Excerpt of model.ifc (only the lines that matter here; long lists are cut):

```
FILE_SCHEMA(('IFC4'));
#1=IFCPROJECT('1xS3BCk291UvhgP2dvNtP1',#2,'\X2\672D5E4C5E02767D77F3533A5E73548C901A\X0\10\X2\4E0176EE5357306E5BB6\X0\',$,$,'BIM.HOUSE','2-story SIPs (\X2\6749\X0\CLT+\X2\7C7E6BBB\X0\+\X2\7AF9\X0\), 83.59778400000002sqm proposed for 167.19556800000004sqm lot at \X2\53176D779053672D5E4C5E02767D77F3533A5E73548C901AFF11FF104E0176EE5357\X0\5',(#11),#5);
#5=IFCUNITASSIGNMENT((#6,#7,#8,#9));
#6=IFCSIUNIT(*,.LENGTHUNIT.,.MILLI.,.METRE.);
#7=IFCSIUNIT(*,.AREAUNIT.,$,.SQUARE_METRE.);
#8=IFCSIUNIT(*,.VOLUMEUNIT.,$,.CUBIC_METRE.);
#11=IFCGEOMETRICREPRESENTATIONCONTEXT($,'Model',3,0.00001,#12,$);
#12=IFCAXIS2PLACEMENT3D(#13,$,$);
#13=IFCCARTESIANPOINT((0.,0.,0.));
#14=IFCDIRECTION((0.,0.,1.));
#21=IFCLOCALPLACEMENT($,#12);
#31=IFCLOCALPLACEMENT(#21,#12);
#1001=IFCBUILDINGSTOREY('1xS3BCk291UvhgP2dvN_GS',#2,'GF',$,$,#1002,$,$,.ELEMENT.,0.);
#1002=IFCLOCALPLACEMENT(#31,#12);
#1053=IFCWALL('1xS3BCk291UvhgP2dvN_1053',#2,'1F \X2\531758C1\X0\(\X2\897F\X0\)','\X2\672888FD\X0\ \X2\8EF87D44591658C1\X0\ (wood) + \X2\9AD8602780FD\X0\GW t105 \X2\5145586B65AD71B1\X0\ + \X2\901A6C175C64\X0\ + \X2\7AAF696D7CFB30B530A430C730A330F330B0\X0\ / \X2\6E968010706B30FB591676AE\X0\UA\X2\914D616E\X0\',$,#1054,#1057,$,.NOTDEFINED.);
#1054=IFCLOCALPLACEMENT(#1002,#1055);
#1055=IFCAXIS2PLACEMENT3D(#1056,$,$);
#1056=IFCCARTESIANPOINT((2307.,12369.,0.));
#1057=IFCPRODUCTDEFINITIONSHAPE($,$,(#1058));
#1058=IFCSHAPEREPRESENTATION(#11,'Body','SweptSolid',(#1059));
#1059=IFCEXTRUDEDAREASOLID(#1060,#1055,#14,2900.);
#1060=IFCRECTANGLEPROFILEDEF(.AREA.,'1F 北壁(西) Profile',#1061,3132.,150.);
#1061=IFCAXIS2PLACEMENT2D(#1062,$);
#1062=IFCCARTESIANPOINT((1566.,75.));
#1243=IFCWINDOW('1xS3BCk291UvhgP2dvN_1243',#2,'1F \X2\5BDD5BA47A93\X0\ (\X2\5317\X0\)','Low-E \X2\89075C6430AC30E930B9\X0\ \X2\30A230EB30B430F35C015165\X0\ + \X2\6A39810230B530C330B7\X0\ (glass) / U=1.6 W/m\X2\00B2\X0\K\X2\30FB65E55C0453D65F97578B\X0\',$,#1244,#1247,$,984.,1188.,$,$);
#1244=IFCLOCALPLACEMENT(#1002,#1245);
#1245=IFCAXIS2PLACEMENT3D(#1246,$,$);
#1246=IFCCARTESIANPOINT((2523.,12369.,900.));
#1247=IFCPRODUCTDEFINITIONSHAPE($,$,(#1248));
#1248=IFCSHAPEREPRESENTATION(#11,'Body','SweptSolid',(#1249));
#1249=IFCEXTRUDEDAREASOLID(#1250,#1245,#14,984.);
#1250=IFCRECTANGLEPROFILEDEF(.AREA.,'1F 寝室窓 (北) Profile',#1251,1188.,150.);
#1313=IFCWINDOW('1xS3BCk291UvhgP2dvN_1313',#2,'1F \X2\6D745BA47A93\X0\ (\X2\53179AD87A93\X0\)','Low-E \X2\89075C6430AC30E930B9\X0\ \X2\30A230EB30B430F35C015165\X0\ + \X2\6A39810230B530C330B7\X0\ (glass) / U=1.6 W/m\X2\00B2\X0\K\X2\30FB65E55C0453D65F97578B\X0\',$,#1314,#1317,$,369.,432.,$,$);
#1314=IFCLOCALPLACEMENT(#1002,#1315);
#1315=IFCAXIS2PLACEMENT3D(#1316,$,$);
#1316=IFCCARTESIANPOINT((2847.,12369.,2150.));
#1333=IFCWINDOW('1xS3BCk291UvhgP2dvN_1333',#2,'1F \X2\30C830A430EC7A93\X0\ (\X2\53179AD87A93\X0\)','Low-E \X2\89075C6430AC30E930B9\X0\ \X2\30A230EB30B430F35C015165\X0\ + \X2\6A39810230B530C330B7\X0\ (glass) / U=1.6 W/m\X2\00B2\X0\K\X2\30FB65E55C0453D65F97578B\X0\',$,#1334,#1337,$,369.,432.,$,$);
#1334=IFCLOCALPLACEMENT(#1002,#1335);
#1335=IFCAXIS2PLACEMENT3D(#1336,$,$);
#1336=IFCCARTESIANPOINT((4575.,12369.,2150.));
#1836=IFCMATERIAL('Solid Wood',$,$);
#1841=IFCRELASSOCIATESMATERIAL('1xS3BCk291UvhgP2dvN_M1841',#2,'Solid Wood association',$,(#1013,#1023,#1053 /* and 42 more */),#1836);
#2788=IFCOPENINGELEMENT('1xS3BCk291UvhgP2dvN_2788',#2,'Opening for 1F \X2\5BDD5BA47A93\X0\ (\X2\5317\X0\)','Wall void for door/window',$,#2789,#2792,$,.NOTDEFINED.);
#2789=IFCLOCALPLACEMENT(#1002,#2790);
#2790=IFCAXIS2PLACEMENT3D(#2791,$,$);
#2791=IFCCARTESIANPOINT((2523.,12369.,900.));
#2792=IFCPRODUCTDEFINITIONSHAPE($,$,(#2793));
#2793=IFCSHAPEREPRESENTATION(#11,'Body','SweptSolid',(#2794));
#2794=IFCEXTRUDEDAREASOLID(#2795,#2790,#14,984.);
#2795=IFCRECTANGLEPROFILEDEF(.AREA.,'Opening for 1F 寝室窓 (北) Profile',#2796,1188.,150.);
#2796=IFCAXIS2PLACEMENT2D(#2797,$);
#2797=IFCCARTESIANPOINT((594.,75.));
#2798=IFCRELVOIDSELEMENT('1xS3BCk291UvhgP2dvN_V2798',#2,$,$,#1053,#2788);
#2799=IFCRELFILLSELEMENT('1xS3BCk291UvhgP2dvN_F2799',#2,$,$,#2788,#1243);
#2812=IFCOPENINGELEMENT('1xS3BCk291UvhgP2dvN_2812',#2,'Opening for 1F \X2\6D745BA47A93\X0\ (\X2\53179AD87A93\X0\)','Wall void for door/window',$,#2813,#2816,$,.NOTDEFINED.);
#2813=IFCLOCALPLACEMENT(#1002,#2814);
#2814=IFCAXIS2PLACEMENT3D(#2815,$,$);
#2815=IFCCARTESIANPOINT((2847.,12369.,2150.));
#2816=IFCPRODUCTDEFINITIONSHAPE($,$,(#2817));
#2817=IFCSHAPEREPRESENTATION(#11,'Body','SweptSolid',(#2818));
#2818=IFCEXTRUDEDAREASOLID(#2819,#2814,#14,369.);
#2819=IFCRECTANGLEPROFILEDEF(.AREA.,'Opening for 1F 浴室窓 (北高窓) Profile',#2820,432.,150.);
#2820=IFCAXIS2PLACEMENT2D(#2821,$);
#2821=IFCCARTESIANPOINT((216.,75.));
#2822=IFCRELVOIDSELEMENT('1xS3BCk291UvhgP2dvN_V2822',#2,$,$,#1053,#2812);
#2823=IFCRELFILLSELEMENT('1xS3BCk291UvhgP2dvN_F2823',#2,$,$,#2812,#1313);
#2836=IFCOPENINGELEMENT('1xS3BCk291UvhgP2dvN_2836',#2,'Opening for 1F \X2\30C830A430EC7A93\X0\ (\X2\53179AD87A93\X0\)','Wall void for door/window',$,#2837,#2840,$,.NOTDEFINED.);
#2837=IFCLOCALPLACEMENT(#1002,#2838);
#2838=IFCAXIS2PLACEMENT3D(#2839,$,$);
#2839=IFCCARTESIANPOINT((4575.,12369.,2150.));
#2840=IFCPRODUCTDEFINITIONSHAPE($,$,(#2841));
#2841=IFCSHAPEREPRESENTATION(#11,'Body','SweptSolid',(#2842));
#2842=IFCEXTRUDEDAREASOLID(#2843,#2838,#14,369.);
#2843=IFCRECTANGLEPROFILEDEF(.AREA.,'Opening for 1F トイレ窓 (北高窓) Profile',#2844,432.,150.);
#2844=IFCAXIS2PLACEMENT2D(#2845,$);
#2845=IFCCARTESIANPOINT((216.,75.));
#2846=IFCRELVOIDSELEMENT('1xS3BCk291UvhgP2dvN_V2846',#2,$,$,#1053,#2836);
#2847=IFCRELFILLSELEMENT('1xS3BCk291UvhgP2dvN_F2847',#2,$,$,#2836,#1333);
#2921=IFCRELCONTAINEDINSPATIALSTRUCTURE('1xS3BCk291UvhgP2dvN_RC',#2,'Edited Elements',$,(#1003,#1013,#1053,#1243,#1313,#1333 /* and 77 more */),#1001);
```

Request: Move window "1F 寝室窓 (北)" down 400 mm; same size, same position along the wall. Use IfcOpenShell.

```python
import numpy as np
import ifcopenshell
import ifcopenshell.api.geometry
import ifcopenshell.util.placement
import ifcopenshell.util.unit

model = ifcopenshell.open("model.ifc")
unit_scale = ifcopenshell.util.unit.calculate_unit_scale(model)

window = model.by_id(1243)
opening = window.FillsVoids[0].RelatingOpeningElement
dz = -0.4 / unit_scale

shift = np.array([0.0, 0.0, dz])
# The window is not placed relative to its opening, so move both.
for product in (opening, window):
    matrix = ifcopenshell.util.placement.get_local_placement(product.ObjectPlacement)
    matrix[:3, 3] += shift
    ifcopenshell.api.geometry.edit_object_placement(model, product=product, matrix=matrix, is_si=False)

print(f"moved by {dz * unit_scale:+.3f} m")

model.write("model_edited.ifc")
```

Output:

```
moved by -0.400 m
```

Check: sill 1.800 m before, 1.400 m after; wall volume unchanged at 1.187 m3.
